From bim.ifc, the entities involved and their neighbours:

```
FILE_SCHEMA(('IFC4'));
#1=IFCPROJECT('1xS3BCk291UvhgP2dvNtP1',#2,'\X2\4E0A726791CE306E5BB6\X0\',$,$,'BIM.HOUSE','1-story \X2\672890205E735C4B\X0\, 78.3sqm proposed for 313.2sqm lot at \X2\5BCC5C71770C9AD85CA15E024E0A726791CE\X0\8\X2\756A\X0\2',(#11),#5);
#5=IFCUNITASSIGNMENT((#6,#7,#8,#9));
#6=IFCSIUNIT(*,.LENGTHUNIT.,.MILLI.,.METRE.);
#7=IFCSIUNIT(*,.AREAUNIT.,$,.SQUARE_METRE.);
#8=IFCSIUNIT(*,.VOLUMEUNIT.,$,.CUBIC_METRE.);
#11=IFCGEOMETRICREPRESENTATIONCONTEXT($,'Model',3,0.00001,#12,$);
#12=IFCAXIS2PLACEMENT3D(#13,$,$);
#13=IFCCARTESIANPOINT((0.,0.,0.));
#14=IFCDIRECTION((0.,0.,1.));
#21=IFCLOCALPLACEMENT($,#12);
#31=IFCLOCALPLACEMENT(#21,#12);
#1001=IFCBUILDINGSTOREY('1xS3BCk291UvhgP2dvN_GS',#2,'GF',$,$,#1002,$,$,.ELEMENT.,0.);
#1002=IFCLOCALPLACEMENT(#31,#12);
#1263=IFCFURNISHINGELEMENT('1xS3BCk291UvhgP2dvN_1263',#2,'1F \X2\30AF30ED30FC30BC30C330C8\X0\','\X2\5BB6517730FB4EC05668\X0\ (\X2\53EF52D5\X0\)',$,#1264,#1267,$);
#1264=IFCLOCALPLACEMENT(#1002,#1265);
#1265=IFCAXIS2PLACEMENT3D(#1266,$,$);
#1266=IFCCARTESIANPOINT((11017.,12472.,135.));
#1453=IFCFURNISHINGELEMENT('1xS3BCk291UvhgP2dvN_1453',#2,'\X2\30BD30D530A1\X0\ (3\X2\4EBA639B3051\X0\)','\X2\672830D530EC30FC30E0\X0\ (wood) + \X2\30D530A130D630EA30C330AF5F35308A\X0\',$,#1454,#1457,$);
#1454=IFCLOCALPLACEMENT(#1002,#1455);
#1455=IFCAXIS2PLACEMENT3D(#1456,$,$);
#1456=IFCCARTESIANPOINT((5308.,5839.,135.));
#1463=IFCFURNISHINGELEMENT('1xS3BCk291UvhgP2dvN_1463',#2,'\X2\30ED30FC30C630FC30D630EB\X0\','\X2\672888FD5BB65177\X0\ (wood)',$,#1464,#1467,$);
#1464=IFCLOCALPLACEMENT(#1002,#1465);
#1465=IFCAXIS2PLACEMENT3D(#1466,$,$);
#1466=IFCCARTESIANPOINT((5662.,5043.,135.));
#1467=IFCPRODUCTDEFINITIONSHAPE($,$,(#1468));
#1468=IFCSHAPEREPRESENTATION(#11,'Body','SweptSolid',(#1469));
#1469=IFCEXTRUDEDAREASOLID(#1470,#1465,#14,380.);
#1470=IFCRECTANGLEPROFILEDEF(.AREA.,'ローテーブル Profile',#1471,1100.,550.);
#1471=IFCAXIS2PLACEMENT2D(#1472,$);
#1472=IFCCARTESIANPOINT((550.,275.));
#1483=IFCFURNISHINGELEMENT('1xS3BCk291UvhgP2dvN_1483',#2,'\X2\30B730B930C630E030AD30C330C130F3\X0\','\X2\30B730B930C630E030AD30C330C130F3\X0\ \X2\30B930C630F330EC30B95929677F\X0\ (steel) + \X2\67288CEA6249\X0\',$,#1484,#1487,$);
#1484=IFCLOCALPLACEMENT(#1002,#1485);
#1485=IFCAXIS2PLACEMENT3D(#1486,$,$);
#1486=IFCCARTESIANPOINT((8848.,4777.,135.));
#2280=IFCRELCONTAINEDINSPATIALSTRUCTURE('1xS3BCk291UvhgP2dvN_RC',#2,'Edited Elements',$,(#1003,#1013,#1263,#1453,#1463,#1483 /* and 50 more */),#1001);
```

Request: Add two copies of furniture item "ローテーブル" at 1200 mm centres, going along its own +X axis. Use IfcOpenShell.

```python
import ifcopenshell
import ifcopenshell.api.geometry
import ifcopenshell.api.root
import ifcopenshell.util.element
import ifcopenshell.util.placement

model = ifcopenshell.open("bim.ifc")


def reuse_history(source, copy):
    """copy_class also copies each property set's owner history, people and application; keep the originals."""
    for rel in copy.IsDefinedBy:
        if rel.is_a("IfcRelDefinesByProperties") and (history := rel.RelatingPropertyDefinition.OwnerHistory):
            rel.RelatingPropertyDefinition.OwnerHistory = source.OwnerHistory
            ifcopenshell.util.element.remove_deep2(model, history)


source = model.by_guid("1xS3BCk291UvhgP2dvN_1463")
base = ifcopenshell.util.placement.get_local_placement(source.ObjectPlacement)
step = base[:3, 0] * 1200.0

for i in range(1, 3):
    copy = ifcopenshell.api.root.copy_class(model, product=source)
    copy.Representation = ifcopenshell.util.element.copy_deep(
        model, source.Representation, exclude=["IfcGeometricRepresentationContext", "IfcRepresentationMap"]
    )
    reuse_history(source, copy)
    matrix = base.copy()
    matrix[:3, 3] += i * step
    print("added at", matrix[:3, 3].round(3) + 0.0)
    ifcopenshell.api.geometry.edit_object_placement(model, product=copy, matrix=matrix, is_si=False)

model.write("bim-out.ifc")
```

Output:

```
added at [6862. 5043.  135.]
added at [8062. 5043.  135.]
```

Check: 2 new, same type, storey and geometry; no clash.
